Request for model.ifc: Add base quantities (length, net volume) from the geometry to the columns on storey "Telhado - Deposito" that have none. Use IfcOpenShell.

First a look at what the model holds.

```python
import ifcopenshell
import ifcopenshell.util.element
import ifcopenshell.util.unit

model = ifcopenshell.open("model.ifc")
print(model.schema)
for unit_type in ("LENGTHUNIT", "AREAUNIT", "VOLUMEUNIT"):
    print(unit_type, ifcopenshell.util.unit.calculate_unit_scale(model, unit_type))
storey = next(s for s in model.by_type("IfcBuildingStorey") if s.Name == "Telhado - Deposito")
columns = [e for e in ifcopenshell.util.element.get_decomposition(storey) if e.is_a("IfcColumn")]
for e in sorted(columns, key=lambda e: e.id()):
    print(e.id(), e.is_a(), e.Name, list(ifcopenshell.util.element.get_psets(e, qtos_only=True)), sep=" | ")
```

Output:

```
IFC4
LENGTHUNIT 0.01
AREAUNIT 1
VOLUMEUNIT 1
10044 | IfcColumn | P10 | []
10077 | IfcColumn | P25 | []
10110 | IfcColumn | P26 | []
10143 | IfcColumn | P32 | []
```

```python
import ifcopenshell
import ifcopenshell.api.pset
import ifcopenshell.geom
import ifcopenshell.util.element
import ifcopenshell.util.shape
import ifcopenshell.util.unit

model = ifcopenshell.open("model.ifc")
unit_scale = ifcopenshell.util.unit.calculate_unit_scale(model)
volume_scale = ifcopenshell.util.unit.calculate_unit_scale(model, "VOLUMEUNIT")
settings = ifcopenshell.geom.settings()

storey = next(s for s in model.by_type("IfcBuildingStorey") if s.Name == "Telhado - Deposito")
columns = [e for e in ifcopenshell.util.element.get_decomposition(storey) if e.is_a("IfcColumn")]

for e in sorted(columns, key=lambda e: e.id()):
    if ifcopenshell.util.element.get_psets(e, qtos_only=True, should_inherit=False):
        continue
    # Geometry comes back in metres, in the element's own axes.
    shape = ifcopenshell.geom.create_shape(settings, e)
    values = {
        "Length": ifcopenshell.util.shape.get_z(shape.geometry) / unit_scale,
        "NetVolume": ifcopenshell.util.shape.get_volume(shape.geometry) / volume_scale,
    }
    qto = ifcopenshell.api.pset.add_qto(model, product=e, name="Qto_ColumnBaseQuantities")
    ifcopenshell.api.pset.edit_qto(model, qto=qto, properties=values)
    print(e.id(), {k: round(v, 3) for k, v in values.items()})

model.write("model_v2.ifc")
```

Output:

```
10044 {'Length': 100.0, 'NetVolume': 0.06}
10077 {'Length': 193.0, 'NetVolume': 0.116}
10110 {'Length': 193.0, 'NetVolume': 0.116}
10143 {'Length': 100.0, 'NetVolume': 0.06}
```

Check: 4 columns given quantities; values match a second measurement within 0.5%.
